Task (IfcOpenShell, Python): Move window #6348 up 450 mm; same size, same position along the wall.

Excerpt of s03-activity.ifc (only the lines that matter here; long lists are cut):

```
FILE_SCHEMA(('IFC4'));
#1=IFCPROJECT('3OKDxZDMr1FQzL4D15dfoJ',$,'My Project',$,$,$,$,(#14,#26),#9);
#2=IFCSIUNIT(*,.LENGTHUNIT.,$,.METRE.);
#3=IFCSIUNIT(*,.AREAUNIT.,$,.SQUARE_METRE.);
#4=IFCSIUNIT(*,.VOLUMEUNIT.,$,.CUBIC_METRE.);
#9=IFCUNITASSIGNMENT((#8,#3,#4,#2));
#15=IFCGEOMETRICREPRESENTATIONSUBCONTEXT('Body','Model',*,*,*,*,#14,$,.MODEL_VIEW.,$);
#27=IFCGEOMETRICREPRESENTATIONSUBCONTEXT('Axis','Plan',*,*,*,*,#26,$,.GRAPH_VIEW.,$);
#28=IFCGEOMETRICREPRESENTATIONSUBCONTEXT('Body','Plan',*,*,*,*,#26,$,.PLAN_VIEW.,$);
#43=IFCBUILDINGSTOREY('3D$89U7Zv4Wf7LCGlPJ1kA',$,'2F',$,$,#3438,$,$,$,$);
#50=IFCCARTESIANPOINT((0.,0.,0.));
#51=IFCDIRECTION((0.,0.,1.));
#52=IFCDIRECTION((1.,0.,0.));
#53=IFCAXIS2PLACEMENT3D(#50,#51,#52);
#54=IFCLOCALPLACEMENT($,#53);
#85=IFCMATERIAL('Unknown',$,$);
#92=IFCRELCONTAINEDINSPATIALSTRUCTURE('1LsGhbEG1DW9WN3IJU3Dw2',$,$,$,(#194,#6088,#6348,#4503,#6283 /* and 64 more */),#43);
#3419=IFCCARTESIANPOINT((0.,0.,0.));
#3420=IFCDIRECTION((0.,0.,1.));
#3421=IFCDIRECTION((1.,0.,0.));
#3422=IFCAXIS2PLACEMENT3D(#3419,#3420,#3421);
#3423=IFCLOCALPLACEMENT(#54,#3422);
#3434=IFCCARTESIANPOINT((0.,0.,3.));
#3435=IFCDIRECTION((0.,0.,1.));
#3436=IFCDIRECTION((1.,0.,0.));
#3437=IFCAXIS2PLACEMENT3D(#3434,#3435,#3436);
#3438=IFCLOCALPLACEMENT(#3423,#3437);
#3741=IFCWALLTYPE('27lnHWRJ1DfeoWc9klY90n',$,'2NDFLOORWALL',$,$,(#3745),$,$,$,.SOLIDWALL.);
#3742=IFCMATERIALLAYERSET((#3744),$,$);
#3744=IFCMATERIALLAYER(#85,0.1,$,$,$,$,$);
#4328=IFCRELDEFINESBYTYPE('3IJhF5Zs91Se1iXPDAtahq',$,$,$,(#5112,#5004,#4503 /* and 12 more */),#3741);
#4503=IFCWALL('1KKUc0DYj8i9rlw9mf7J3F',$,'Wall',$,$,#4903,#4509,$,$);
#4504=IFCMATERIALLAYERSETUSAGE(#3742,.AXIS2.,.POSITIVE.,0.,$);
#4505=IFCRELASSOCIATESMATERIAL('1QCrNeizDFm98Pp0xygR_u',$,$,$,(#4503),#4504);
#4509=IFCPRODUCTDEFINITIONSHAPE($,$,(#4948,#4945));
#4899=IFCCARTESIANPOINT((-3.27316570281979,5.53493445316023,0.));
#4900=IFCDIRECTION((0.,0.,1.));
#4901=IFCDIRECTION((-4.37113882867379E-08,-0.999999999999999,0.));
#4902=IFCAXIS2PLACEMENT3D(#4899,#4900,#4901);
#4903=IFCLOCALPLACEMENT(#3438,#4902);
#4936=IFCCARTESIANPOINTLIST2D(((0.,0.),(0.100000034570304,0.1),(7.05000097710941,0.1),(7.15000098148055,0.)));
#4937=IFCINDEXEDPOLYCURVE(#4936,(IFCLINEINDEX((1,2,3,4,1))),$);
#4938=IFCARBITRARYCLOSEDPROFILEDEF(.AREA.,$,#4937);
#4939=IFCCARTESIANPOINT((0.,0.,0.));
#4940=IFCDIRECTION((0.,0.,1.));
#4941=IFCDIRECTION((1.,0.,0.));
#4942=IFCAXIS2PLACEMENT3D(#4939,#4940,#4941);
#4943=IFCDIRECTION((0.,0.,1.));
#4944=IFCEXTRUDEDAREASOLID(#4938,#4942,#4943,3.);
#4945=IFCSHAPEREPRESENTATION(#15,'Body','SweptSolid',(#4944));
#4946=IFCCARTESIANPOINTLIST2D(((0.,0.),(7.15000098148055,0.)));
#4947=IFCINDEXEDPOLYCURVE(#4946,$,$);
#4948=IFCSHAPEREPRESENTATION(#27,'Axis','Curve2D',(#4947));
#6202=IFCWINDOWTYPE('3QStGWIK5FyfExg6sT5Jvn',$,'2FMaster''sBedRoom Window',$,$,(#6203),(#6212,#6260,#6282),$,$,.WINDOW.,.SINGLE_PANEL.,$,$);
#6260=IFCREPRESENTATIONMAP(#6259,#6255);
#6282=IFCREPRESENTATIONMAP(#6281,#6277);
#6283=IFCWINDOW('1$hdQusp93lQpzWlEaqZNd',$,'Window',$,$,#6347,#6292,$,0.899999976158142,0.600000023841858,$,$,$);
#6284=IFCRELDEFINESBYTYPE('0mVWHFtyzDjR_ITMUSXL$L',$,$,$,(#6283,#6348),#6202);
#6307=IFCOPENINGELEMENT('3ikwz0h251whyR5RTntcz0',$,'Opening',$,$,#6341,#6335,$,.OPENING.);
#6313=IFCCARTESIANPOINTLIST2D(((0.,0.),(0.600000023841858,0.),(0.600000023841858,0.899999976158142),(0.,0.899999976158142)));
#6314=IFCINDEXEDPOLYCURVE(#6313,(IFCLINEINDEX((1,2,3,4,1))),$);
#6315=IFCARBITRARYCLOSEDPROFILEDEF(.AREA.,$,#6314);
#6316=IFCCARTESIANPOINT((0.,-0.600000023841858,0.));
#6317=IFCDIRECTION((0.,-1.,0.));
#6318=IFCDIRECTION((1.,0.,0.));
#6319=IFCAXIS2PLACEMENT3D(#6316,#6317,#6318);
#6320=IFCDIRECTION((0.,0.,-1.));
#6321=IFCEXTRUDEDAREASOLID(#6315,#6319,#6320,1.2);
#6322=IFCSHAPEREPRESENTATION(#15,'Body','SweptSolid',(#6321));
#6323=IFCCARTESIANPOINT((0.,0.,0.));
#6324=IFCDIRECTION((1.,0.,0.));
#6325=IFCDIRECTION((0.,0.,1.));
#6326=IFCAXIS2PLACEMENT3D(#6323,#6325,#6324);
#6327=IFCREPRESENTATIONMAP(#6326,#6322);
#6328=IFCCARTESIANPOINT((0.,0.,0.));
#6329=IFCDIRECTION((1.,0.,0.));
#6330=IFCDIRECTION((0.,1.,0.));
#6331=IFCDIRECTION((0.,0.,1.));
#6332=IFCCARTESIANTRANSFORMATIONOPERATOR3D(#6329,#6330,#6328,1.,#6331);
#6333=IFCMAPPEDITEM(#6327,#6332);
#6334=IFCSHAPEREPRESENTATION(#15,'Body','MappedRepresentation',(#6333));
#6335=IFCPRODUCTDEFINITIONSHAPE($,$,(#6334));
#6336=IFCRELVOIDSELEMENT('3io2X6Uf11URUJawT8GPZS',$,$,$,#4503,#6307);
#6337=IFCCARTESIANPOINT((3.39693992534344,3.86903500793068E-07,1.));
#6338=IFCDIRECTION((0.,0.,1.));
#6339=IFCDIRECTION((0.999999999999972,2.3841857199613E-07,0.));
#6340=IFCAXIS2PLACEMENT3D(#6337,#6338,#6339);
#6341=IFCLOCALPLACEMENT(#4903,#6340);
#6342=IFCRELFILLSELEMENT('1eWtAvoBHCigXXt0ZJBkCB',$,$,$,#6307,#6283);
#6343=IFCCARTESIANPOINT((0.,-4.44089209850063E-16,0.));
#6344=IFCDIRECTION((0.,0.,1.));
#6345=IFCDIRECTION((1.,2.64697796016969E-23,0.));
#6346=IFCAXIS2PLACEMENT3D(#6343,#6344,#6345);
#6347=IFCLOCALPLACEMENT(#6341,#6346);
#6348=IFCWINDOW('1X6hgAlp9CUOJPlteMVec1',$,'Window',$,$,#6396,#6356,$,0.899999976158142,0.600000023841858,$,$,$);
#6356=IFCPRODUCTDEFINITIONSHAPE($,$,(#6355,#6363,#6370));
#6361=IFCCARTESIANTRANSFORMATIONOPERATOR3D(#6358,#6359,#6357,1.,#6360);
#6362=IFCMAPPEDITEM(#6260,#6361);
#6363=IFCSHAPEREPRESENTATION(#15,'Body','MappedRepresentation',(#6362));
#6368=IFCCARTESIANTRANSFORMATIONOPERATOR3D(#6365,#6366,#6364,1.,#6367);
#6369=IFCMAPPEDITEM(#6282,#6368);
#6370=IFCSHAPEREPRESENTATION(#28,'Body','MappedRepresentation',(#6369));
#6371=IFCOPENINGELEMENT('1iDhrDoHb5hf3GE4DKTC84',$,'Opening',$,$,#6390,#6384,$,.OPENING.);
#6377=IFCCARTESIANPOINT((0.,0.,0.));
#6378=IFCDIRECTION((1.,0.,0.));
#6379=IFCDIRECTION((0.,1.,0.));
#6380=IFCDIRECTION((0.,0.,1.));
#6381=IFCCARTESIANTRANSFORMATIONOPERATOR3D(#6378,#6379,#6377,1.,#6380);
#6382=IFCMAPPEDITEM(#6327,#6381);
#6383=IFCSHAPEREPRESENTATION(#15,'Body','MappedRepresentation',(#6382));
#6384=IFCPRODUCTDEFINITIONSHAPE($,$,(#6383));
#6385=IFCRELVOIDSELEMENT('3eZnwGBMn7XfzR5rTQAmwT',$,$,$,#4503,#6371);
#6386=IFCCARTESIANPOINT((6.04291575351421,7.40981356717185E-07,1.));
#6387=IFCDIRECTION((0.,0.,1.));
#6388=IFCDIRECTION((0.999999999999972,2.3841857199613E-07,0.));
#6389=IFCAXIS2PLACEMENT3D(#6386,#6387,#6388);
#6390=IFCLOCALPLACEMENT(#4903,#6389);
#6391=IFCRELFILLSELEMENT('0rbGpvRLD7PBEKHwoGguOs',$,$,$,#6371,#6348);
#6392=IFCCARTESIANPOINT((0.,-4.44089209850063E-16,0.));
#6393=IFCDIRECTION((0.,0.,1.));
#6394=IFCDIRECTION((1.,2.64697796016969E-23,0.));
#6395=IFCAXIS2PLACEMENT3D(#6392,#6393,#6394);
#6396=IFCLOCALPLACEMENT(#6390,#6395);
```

```python
import numpy as np
import ifcopenshell
import ifcopenshell.api.geometry
import ifcopenshell.util.placement
import ifcopenshell.util.unit

model = ifcopenshell.open("s03-activity.ifc")
unit_scale = ifcopenshell.util.unit.calculate_unit_scale(model)

window = model.by_guid("1X6hgAlp9CUOJPlteMVec1")
opening = window.FillsVoids[0].RelatingOpeningElement
dz = 0.45 / unit_scale

shift = np.array([0.0, 0.0, dz])
# The window is placed relative to its opening, so it follows when the opening moves.
matrix = ifcopenshell.util.placement.get_local_placement(opening.ObjectPlacement)
matrix[:3, 3] += shift
ifcopenshell.api.geometry.edit_object_placement(
    model, product=opening, matrix=matrix, is_si=False, should_transform_children=True
)

print(f"moved by {dz * unit_scale:+.3f} m")

model.write("s03-activity_rev.ifc")
```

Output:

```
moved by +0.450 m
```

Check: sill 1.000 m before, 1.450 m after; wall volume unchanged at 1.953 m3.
